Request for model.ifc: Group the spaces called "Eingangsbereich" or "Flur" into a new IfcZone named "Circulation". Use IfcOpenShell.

First a look at what the model holds.

```python
import ifcopenshell

model = ifcopenshell.open("model.ifc")
print(model.schema)
seen = {}
for space in model.by_type("IfcSpace"):
    seen[space.LongName] = seen.get(space.LongName, 0) + 1
for name, count in sorted(seen.items(), key=str):
    print(count, "x", name)
print("zones:", [z.Name for z in model.by_type("IfcZone")][:20])
```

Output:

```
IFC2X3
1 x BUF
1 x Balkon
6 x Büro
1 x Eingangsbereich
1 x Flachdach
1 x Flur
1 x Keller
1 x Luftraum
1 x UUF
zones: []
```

```python
import ifcopenshell
import ifcopenshell.api.group
import ifcopenshell.api.root

model = ifcopenshell.open("model.ifc")

names = {"Eingangsbereich", "Flur"}
spaces = [s for s in model.by_type("IfcSpace") if s.LongName in names]

zone = ifcopenshell.api.root.create_entity(model, ifc_class="IfcZone", name="Circulation")
ifcopenshell.api.group.assign_group(model, products=spaces, group=zone)
print(len(spaces), "spaces in", zone.Name)

model.write("model_v2.ifc")
```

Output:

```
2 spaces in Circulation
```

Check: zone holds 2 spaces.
